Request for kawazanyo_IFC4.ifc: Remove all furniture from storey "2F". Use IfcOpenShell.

First a look at what the model holds.

```python
import ifcopenshell
import ifcopenshell.util.element

model = ifcopenshell.open("kawazanyo_IFC4.ifc")
print(model.schema)
storey = next(s for s in model.by_type("IfcBuildingStorey") if s.Name == "2F")
furniture = [e for e in ifcopenshell.util.element.get_decomposition(storey) if e.is_a("IfcFurnishingElement")]
seen = {}
for e in furniture:
    element_type = ifcopenshell.util.element.get_type(e)
    name = element_type.Name if element_type not in (None, e) else None
    seen[name] = seen.get(name, 0) + 1
for name, count in sorted(seen.items(), key=str):
    print(count, "x", name)
```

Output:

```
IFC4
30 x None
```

```python
import ifcopenshell
import ifcopenshell.api.root
import ifcopenshell.util.element

model = ifcopenshell.open("kawazanyo_IFC4.ifc")

storey = next(s for s in model.by_type("IfcBuildingStorey") if s.Name == "2F")
furniture = [e for e in ifcopenshell.util.element.get_decomposition(storey) if e.is_a("IfcFurnishingElement")]

for e in furniture:
    ifcopenshell.api.root.remove_product(model, product=e)
print(len(furniture), "removed")

model.write("kawazanyo_IFC4_updated.ifc")
```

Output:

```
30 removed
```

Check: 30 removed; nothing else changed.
